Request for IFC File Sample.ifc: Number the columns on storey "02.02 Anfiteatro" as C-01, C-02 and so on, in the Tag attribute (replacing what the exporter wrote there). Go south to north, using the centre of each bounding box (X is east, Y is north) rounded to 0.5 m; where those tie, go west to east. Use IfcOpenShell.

First a look at what the model holds.

```python
import ifcopenshell
import ifcopenshell.util.element
import ifcopenshell.util.placement

model = ifcopenshell.open("IFC File Sample.ifc")
print(model.schema)
storey = next(s for s in model.by_type("IfcBuildingStorey") if s.Name == "02.02 Anfiteatro")
columns = [e for e in ifcopenshell.util.element.get_decomposition(storey) if e.is_a("IfcColumn")]
for e in sorted(columns, key=lambda e: e.id()):
    origin = ifcopenshell.util.placement.get_local_placement(e.ObjectPlacement)[:3, 3]
    print(e.id(), e.Tag, e.Name, origin.round(2) + 0.0, sep=" | ")
```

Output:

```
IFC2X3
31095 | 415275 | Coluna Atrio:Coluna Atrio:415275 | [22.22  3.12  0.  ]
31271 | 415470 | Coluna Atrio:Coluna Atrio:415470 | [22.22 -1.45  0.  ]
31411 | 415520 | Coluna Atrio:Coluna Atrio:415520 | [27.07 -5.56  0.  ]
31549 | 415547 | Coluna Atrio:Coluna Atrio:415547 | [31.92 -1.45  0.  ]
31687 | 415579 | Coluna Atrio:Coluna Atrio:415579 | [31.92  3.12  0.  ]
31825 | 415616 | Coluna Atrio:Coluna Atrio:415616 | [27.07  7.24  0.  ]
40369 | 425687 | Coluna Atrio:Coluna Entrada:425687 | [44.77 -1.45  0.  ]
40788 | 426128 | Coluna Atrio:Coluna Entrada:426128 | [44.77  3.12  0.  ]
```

```python
import ifcopenshell
import ifcopenshell.geom
import ifcopenshell.util.element
import ifcopenshell.util.shape

model = ifcopenshell.open("IFC File Sample.ifc")
settings = ifcopenshell.geom.settings()
settings.set("use-world-coords", True)


def centre(element):
    shape = ifcopenshell.geom.create_shape(settings, element)
    return ifcopenshell.util.shape.get_bbox_centroid(shape.geometry)


storey = next(s for s in model.by_type("IfcBuildingStorey") if s.Name == "02.02 Anfiteatro")
columns = [e for e in ifcopenshell.util.element.get_decomposition(storey) if e.is_a("IfcColumn")]

# Insertion points can sit at a corner or the storey origin, so sort by the geometry (in metres).
centres = {e: centre(e) for e in columns}
columns.sort(key=lambda e: (round(centres[e][1] / 0.5), centres[e][0]))

for i, e in enumerate(columns, start=1):
    number = f"C-{i:02d}"
    e.Tag = number
    print(e.id(), number)

model.write("IFC File Sample_rev.ifc")
```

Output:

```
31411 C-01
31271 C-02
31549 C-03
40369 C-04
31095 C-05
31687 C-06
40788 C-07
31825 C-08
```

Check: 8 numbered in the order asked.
